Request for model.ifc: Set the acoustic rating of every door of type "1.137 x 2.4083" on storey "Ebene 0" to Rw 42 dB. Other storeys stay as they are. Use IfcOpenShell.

First a look at what the model holds.

```python
import ifcopenshell
import ifcopenshell.util.element

model = ifcopenshell.open("model.ifc")
print(model.schema)
storey = next(s for s in model.by_type("IfcBuildingStorey") if s.Name == "Ebene 0")
doors = [e for e in ifcopenshell.util.element.get_decomposition(storey) if e.is_a("IfcDoor")]
seen = {}
for e in doors:
    element_type = ifcopenshell.util.element.get_type(e)
    key = (element_type.Name if element_type != e and element_type else None, ifcopenshell.util.element.get_pset(e, "Pset_DoorCommon", "AcousticRating"))
    seen[key] = seen.get(key, 0) + 1
for (name, value), count in sorted(seen.items(), key=str):
    print(count, "x", name, "|", value)
```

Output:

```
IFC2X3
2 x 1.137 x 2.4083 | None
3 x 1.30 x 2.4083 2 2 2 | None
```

```python
import ifcopenshell
import ifcopenshell.api.pset
import ifcopenshell.util.element

model = ifcopenshell.open("model.ifc")

storey = next(s for s in model.by_type("IfcBuildingStorey") if s.Name == "Ebene 0")
doors = [e for e in ifcopenshell.util.element.get_decomposition(storey) if e.is_a("IfcDoor")]

count = 0
for e in doors:
    element_type = ifcopenshell.util.element.get_type(e)
    if element_type in (None, e) or element_type.Name != "1.137 x 2.4083":
        continue
    # add_pset returns the element's existing set when there is one.
    pset = ifcopenshell.api.pset.add_pset(model, product=e, name="Pset_DoorCommon")
    ifcopenshell.api.pset.edit_pset(model, pset=pset, properties={"AcousticRating": "Rw 42 dB"})
    count += 1

print(count, "doors updated")

model.write("model-out.ifc")
```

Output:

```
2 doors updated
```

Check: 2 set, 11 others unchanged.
